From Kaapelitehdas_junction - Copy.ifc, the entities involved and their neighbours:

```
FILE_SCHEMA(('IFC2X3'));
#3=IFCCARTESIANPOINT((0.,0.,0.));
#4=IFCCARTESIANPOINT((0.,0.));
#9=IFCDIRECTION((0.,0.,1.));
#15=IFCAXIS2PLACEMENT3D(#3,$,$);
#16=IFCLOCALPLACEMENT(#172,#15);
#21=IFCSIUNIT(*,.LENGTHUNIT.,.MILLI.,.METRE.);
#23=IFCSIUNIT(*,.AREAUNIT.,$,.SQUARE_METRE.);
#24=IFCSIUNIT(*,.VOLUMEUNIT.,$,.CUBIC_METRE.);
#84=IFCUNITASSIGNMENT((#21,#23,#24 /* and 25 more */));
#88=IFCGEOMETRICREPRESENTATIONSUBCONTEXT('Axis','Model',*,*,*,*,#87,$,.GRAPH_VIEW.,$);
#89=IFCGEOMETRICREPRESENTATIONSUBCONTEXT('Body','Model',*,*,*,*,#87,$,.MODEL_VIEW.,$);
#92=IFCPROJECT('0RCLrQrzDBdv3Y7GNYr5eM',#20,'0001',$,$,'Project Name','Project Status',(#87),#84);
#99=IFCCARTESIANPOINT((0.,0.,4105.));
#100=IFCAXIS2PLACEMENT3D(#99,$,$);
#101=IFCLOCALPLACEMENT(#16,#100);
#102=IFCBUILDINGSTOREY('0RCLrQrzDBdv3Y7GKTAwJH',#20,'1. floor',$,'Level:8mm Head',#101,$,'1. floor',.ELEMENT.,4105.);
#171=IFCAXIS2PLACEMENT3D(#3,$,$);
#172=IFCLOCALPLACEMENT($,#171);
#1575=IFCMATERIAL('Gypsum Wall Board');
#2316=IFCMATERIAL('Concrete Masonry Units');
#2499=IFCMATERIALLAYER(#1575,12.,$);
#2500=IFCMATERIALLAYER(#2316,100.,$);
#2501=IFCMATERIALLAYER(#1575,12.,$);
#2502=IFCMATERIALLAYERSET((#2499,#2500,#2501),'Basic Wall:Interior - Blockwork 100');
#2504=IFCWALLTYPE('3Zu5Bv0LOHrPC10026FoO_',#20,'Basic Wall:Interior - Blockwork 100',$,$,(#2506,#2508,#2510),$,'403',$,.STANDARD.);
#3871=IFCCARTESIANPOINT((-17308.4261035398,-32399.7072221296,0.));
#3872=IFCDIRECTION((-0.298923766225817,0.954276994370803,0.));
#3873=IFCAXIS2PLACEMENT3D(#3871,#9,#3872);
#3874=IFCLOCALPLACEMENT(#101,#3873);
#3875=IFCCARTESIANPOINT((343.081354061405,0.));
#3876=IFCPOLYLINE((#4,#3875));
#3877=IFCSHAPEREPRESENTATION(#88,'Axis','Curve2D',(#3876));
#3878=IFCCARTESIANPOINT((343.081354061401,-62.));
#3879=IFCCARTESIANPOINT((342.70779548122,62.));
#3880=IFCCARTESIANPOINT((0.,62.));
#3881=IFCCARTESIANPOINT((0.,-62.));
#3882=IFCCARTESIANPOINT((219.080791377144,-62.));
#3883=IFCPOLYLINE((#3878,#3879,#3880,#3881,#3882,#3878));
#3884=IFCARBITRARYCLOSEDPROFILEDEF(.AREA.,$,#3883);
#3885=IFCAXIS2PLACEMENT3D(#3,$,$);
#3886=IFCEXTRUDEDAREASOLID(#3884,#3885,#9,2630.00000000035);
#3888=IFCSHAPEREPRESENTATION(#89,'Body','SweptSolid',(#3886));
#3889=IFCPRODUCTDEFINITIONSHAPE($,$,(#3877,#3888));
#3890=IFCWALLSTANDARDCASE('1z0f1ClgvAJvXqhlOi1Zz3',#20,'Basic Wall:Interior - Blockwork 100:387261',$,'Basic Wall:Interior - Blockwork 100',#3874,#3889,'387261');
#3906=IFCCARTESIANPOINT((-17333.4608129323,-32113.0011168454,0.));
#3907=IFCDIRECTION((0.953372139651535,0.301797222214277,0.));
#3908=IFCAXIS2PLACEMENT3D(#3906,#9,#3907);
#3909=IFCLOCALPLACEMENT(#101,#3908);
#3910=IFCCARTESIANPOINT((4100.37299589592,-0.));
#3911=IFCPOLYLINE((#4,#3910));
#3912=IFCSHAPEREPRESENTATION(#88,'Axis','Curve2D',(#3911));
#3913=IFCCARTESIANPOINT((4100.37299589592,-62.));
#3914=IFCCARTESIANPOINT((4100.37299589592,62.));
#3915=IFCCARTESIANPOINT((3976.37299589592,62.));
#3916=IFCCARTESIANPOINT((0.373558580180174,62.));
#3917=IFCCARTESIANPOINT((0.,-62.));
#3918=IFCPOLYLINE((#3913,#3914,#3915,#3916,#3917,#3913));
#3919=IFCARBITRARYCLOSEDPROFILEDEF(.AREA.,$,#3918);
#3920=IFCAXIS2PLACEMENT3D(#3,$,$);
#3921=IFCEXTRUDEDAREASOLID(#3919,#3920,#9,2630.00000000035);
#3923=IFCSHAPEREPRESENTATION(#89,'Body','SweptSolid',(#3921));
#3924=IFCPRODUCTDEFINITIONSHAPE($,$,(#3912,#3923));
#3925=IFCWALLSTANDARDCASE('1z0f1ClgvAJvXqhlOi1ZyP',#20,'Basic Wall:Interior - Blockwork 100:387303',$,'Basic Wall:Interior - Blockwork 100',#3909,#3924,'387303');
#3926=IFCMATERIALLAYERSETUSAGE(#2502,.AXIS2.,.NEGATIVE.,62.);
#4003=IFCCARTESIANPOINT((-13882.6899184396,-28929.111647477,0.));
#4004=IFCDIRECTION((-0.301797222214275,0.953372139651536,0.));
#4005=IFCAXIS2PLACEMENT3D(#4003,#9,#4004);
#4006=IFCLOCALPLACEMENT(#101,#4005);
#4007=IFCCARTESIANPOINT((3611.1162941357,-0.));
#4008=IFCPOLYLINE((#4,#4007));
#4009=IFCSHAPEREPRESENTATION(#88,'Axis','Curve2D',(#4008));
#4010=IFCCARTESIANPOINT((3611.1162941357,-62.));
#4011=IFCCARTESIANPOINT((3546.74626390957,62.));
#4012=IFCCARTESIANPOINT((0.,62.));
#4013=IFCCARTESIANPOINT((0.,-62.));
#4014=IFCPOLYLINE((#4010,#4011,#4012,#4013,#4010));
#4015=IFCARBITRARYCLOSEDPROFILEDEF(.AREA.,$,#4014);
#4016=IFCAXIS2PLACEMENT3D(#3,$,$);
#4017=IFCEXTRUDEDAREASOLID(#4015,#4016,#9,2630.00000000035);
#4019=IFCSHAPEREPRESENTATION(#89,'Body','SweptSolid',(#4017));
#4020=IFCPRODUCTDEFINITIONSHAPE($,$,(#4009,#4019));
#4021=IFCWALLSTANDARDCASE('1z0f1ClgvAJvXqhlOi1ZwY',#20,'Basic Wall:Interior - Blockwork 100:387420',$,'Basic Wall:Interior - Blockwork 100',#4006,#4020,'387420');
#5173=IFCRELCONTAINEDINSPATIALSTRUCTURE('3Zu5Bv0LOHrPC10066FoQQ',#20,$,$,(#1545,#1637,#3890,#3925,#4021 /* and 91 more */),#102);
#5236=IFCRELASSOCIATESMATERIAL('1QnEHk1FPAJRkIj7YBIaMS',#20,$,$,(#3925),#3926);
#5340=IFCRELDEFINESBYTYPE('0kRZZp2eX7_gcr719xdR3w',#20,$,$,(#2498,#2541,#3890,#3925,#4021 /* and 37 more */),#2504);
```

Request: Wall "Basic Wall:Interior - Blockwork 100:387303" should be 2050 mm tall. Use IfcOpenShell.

```python
import ifcopenshell
import ifcopenshell.geom
import ifcopenshell.util.representation
import ifcopenshell.util.shape
import ifcopenshell.util.unit

model = ifcopenshell.open("Kaapelitehdas_junction - Copy.ifc")
unit_scale = ifcopenshell.util.unit.calculate_unit_scale(model)
settings = ifcopenshell.geom.settings()


def volume(element):
    """Net volume in cubic metres, openings subtracted."""
    shape = ifcopenshell.geom.create_shape(settings, element)
    return ifcopenshell.util.shape.get_volume(shape.geometry)


wall = model.by_id(3925)
before = volume(wall)

body = ifcopenshell.util.representation.get_representation(wall, "Model", "Body")
solid = body.Items[0]
old_height = solid.Depth
solid.Depth = 2.05 / unit_scale
after = volume(wall)

print(f"height {old_height:g} -> {solid.Depth:g}, volume {before:.3f} -> {after:.3f} m3")

model.write("Kaapelitehdas_junction - Copy_v2.ifc")
```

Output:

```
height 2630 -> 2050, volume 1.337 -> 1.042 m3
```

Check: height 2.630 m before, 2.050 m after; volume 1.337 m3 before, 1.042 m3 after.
